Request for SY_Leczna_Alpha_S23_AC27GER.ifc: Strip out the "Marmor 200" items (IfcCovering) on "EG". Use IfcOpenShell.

First a look at what the model holds.

```python
import ifcopenshell
import ifcopenshell.util.element

model = ifcopenshell.open("SY_Leczna_Alpha_S23_AC27GER.ifc")
print(model.schema)
storey = next(s for s in model.by_type("IfcBuildingStorey") if s.Name == "EG")
coverings = [e for e in ifcopenshell.util.element.get_decomposition(storey) if e.is_a("IfcCovering")]
seen = {}
for e in coverings:
    element_type = ifcopenshell.util.element.get_type(e)
    name = element_type.Name if element_type not in (None, e) else None
    seen[name] = seen.get(name, 0) + 1
for name, count in sorted(seen.items(), key=str):
    print(count, "x", name)
```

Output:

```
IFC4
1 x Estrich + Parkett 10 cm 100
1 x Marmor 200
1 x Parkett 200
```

```python
import ifcopenshell
import ifcopenshell.api.root
import ifcopenshell.util.element

model = ifcopenshell.open("SY_Leczna_Alpha_S23_AC27GER.ifc")

storey = next(s for s in model.by_type("IfcBuildingStorey") if s.Name == "EG")
coverings = [e for e in ifcopenshell.util.element.get_decomposition(storey) if e.is_a("IfcCovering")]
targets = [e for e in coverings if (t := ifcopenshell.util.element.get_type(e)) not in (None, e) and t.Name == "Marmor 200"]

for e in targets:
    ifcopenshell.api.root.remove_product(model, product=e)
print(len(targets), "removed")

model.write("SY_Leczna_Alpha_S23_AC27GER_edited.ifc")
```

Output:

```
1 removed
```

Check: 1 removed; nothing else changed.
